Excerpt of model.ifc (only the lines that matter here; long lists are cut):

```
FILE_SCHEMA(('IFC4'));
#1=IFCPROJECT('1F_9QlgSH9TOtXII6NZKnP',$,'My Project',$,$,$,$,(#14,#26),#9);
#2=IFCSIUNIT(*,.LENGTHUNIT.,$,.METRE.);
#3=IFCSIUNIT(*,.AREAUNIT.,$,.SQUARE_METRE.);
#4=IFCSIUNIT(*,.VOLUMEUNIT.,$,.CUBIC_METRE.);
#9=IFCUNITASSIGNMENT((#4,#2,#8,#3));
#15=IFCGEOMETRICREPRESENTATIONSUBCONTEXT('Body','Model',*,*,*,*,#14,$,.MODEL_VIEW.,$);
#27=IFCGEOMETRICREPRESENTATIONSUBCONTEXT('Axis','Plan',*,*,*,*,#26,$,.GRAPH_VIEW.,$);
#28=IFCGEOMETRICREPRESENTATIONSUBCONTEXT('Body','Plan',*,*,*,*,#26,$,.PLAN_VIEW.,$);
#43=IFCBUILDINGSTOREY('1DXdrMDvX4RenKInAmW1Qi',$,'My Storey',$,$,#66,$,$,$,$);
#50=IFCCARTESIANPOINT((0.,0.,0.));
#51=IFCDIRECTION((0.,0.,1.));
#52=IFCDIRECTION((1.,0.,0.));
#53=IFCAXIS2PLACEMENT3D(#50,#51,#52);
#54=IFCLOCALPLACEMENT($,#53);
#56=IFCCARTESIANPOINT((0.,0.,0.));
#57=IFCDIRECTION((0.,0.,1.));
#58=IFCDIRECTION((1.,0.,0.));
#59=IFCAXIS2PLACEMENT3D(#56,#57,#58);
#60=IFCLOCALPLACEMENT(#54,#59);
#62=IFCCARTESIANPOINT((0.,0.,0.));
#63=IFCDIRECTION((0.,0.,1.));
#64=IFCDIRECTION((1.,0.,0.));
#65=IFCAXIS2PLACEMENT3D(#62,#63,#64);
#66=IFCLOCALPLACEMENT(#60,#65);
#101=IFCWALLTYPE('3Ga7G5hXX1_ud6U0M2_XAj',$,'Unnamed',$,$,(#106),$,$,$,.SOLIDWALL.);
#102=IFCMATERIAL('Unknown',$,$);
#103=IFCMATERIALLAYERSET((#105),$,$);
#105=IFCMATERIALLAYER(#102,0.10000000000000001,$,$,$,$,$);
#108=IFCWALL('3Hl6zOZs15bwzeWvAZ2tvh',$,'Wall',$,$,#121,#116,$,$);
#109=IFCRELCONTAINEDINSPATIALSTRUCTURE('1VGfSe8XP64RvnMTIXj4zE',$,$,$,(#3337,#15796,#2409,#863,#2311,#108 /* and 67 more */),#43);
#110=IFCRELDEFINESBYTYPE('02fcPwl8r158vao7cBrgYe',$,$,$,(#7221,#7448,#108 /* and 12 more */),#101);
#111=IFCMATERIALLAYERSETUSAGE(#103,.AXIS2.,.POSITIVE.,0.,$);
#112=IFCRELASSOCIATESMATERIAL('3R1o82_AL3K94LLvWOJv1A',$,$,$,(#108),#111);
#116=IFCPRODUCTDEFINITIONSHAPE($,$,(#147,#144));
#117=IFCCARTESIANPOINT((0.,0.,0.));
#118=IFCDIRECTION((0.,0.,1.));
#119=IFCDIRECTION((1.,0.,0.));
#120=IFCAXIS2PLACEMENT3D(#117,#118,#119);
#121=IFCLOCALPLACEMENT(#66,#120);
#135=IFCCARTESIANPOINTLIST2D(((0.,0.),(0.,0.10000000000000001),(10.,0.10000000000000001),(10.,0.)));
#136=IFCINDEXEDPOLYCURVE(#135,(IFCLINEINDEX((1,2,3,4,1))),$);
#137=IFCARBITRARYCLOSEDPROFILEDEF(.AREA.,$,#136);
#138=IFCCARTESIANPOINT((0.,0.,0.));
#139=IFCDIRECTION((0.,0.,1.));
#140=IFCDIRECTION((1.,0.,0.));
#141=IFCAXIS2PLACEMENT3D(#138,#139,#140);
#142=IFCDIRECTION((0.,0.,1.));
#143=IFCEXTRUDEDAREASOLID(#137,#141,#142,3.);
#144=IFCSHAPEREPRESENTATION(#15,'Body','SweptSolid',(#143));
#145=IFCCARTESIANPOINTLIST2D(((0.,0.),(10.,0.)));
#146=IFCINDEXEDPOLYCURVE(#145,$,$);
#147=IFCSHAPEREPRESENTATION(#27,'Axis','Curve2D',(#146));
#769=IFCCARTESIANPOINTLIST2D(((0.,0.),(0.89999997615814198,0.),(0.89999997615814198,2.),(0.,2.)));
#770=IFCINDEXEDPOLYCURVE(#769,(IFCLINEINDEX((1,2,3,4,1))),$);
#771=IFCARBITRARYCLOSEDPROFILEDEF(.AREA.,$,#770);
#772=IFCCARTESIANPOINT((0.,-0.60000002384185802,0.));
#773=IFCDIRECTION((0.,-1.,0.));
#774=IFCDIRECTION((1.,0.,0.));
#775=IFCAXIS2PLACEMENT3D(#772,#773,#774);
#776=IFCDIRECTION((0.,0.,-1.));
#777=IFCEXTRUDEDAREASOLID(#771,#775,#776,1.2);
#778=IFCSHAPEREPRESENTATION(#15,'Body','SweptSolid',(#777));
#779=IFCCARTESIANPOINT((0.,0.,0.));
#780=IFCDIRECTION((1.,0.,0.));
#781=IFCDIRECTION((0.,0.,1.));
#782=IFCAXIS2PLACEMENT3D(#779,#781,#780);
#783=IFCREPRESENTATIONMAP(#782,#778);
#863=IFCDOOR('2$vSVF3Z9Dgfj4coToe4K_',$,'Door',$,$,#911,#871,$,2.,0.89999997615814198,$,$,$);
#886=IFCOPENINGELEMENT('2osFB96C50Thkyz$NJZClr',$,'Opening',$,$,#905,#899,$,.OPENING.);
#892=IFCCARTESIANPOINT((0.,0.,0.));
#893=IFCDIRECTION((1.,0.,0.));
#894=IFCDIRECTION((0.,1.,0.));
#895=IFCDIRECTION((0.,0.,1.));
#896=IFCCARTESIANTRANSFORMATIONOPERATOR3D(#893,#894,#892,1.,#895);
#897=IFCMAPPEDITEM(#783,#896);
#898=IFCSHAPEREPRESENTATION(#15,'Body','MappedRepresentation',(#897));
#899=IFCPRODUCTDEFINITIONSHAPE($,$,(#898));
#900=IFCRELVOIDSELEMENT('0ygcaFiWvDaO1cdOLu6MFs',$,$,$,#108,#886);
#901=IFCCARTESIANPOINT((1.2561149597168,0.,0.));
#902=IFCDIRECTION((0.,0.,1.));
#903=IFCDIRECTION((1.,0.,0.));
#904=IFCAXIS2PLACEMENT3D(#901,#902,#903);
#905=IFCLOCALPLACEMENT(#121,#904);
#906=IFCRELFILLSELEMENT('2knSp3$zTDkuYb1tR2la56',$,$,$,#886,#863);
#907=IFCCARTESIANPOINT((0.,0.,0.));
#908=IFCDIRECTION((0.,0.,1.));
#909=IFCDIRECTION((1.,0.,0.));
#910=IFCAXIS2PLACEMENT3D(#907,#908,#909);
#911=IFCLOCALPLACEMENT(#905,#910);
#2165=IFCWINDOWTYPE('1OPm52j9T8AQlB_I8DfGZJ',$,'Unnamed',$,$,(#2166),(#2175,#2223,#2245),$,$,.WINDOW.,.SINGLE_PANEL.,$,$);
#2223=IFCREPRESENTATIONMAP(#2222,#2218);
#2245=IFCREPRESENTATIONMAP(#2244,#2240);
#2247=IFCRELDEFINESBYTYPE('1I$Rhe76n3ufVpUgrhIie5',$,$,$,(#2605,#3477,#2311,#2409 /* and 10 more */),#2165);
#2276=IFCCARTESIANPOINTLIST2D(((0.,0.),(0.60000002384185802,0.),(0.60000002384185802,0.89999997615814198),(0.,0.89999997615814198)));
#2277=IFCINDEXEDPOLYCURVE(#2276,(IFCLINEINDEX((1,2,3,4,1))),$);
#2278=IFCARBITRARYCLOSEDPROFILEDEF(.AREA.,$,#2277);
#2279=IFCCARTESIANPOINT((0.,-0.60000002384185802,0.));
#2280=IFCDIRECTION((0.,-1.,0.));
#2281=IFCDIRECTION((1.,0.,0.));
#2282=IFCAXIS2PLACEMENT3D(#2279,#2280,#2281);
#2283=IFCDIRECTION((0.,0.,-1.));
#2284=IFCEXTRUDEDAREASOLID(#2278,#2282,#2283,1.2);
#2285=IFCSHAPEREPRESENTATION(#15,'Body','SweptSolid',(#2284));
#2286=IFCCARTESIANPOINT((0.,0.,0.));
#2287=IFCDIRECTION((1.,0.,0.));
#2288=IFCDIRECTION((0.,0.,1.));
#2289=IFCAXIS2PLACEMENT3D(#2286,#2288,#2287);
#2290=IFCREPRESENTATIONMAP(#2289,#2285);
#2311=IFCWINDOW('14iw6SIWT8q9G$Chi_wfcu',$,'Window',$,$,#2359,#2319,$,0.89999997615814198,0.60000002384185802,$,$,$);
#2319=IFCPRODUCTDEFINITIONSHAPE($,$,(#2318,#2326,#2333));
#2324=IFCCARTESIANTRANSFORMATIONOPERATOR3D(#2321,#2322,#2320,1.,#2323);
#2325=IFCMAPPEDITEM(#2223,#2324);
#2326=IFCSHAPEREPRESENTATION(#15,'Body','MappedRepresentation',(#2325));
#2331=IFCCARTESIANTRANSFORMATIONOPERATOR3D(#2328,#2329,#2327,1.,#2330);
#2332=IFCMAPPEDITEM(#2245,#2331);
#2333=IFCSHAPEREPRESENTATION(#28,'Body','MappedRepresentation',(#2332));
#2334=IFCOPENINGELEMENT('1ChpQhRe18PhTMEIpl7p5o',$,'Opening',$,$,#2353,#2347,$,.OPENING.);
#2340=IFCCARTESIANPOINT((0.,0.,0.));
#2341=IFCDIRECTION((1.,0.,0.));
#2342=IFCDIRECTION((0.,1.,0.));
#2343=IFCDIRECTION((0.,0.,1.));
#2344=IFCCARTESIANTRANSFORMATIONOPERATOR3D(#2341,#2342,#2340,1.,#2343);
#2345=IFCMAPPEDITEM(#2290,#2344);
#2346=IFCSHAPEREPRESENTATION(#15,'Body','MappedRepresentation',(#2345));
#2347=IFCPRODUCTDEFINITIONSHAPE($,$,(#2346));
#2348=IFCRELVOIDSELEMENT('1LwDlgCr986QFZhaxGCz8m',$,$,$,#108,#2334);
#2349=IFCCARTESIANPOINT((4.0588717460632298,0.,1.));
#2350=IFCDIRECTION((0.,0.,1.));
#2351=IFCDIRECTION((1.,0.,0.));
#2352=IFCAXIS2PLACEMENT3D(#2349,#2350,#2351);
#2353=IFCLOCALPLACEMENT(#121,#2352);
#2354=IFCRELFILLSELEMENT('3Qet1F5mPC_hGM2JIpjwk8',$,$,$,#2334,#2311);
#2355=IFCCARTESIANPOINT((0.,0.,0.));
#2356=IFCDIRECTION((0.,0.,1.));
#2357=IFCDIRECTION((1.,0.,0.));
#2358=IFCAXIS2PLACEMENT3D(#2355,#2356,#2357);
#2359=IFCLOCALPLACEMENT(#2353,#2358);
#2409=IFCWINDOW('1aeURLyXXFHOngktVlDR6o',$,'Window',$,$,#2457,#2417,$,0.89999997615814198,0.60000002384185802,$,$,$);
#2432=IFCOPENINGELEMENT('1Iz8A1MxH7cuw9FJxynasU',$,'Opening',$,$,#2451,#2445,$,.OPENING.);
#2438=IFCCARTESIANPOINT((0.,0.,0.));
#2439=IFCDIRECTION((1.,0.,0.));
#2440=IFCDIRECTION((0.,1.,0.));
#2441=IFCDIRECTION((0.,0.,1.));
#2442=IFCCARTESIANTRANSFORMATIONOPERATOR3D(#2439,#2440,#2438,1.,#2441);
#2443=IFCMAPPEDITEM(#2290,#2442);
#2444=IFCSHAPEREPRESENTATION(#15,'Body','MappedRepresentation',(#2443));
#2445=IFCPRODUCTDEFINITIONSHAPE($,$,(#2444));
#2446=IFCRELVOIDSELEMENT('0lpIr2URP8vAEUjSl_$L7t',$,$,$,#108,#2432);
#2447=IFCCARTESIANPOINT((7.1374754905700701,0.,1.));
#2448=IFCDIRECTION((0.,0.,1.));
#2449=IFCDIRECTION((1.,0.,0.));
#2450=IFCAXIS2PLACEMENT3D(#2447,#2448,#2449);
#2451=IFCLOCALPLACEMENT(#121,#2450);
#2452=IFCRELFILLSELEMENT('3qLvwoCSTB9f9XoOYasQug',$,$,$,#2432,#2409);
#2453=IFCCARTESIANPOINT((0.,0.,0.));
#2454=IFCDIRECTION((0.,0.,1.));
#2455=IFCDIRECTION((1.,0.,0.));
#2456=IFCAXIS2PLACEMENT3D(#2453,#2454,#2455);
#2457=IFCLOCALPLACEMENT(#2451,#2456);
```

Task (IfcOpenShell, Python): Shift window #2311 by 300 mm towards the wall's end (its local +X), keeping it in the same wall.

```python
import ifcopenshell
import ifcopenshell.api.geometry
import ifcopenshell.util.placement
import ifcopenshell.util.unit

model = ifcopenshell.open("model.ifc")
unit_scale = ifcopenshell.util.unit.calculate_unit_scale(model)

window = model.by_guid("14iw6SIWT8q9G$Chi_wfcu")
opening = window.FillsVoids[0].RelatingOpeningElement
wall = opening.VoidsElements[0].RelatingBuildingElement

wall_matrix = ifcopenshell.util.placement.get_local_placement(wall.ObjectPlacement)
shift = wall_matrix[:3, 0] * 0.3 / unit_scale
before = ifcopenshell.util.placement.get_local_placement(window.ObjectPlacement)[:3, 3].copy()

# The window is placed relative to its opening, so it follows when the opening moves.
matrix = ifcopenshell.util.placement.get_local_placement(opening.ObjectPlacement)
matrix[:3, 3] += shift
ifcopenshell.api.geometry.edit_object_placement(
    model, product=opening, matrix=matrix, is_si=False, should_transform_children=True
)

after = ifcopenshell.util.placement.get_local_placement(window.ObjectPlacement)[:3, 3]
print("window moved by", (after - before).round(3) + 0.0)

model.write("model_rev.ifc")
```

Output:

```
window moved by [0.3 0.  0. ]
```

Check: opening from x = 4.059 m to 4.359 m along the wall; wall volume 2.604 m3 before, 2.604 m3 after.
